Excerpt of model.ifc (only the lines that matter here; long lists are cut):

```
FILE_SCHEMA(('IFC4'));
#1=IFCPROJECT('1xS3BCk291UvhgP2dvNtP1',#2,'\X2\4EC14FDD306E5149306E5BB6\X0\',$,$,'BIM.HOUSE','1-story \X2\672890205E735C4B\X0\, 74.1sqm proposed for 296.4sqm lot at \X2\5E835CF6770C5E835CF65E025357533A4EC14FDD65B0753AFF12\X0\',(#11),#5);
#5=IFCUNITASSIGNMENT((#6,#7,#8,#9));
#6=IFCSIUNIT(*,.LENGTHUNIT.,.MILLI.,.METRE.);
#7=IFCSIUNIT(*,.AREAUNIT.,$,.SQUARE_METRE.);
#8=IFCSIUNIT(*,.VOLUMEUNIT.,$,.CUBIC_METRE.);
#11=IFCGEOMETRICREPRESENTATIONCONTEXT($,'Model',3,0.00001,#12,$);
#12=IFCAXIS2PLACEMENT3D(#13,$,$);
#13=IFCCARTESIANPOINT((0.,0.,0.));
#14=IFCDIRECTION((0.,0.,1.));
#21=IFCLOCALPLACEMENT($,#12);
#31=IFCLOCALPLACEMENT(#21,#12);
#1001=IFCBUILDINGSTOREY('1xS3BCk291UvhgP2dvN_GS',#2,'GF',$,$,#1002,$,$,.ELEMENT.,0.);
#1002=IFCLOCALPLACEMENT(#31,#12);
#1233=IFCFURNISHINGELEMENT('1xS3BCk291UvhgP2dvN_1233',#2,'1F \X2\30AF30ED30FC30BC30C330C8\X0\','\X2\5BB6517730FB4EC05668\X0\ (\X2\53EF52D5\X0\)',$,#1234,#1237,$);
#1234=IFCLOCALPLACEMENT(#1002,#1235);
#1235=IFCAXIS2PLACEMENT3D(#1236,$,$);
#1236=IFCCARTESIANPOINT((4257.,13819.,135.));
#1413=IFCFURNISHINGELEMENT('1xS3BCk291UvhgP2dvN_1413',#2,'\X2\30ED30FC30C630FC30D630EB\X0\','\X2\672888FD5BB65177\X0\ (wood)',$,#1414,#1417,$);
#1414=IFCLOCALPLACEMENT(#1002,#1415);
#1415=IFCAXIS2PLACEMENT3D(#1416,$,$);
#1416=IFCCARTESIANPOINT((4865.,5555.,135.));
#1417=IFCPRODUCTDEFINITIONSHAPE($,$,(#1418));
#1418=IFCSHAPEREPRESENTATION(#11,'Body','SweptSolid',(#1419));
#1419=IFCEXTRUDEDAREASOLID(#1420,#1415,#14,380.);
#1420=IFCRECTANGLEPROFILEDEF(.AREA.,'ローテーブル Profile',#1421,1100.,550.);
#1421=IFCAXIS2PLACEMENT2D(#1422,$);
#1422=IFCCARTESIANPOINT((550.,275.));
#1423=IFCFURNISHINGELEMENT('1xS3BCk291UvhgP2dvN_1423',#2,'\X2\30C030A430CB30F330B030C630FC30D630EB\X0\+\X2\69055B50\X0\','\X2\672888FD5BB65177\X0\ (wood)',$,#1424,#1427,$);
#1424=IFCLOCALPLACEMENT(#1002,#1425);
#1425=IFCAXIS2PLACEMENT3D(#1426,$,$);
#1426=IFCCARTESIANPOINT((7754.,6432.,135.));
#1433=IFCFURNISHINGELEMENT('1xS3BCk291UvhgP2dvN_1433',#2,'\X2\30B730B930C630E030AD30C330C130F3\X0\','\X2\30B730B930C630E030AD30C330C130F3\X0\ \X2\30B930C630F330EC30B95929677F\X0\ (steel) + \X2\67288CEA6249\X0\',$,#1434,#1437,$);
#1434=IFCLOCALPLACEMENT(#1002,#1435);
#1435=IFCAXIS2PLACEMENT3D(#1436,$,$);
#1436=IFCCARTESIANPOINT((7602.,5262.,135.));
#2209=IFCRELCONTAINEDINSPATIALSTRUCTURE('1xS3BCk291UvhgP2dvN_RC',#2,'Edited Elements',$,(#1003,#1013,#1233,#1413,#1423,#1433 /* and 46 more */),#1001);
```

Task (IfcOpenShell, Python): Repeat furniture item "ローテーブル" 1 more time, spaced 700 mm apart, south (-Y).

```python
import numpy as np
import ifcopenshell
import ifcopenshell.api.geometry
import ifcopenshell.api.root
import ifcopenshell.util.element
import ifcopenshell.util.placement
import ifcopenshell.util.unit

model = ifcopenshell.open("model.ifc")
unit_scale = ifcopenshell.util.unit.calculate_unit_scale(model)


def reuse_history(source, copy):
    """copy_class also copies each property set's owner history, people and application; keep the originals."""
    for rel in copy.IsDefinedBy:
        if rel.is_a("IfcRelDefinesByProperties") and (history := rel.RelatingPropertyDefinition.OwnerHistory):
            rel.RelatingPropertyDefinition.OwnerHistory = source.OwnerHistory
            ifcopenshell.util.element.remove_deep2(model, history)


source = model.by_guid("1xS3BCk291UvhgP2dvN_1413")
base = ifcopenshell.util.placement.get_local_placement(source.ObjectPlacement)
step = np.array([0.0, -1.0, 0.0]) * 0.7 / unit_scale

for i in range(1, 2):
    copy = ifcopenshell.api.root.copy_class(model, product=source)
    copy.Representation = ifcopenshell.util.element.copy_deep(
        model, source.Representation, exclude=["IfcGeometricRepresentationContext", "IfcRepresentationMap"]
    )
    reuse_history(source, copy)
    matrix = base.copy()
    matrix[:3, 3] += i * step
    print("added at", matrix[:3, 3].round(3) + 0.0)
    ifcopenshell.api.geometry.edit_object_placement(model, product=copy, matrix=matrix, is_si=False)

model.write("model-out.ifc")
```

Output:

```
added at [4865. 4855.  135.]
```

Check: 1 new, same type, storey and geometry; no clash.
